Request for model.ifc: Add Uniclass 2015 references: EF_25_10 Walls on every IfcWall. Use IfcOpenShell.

First a look at what the model holds.

```python
import ifcopenshell

model = ifcopenshell.open("model.ifc")
print(model.schema)
print("classifications:", [c.Name for c in model.by_type("IfcClassification")])
for ifc_class in ("IfcDoor", "IfcRoof", "IfcStair", "IfcWall", "IfcWindow"):
    print(ifc_class, len(model.by_type(ifc_class)))
```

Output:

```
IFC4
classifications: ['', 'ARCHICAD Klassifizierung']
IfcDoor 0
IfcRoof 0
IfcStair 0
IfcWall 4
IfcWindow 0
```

```python
import ifcopenshell
import ifcopenshell.api.classification

model = ifcopenshell.open("model.ifc")

system = ifcopenshell.api.classification.add_classification(model, classification="Uniclass 2015")

codes = {
    "IfcWall": ("EF_25_10", "Walls"),
}
for ifc_class, (code, name) in codes.items():
    products = model.by_type(ifc_class)
    ifcopenshell.api.classification.add_reference(
        model, products=products, classification=system, identification=code, name=name
    )
    print(code, len(products))

model.write("model_v2.ifc")
```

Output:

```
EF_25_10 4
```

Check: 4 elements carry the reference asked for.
